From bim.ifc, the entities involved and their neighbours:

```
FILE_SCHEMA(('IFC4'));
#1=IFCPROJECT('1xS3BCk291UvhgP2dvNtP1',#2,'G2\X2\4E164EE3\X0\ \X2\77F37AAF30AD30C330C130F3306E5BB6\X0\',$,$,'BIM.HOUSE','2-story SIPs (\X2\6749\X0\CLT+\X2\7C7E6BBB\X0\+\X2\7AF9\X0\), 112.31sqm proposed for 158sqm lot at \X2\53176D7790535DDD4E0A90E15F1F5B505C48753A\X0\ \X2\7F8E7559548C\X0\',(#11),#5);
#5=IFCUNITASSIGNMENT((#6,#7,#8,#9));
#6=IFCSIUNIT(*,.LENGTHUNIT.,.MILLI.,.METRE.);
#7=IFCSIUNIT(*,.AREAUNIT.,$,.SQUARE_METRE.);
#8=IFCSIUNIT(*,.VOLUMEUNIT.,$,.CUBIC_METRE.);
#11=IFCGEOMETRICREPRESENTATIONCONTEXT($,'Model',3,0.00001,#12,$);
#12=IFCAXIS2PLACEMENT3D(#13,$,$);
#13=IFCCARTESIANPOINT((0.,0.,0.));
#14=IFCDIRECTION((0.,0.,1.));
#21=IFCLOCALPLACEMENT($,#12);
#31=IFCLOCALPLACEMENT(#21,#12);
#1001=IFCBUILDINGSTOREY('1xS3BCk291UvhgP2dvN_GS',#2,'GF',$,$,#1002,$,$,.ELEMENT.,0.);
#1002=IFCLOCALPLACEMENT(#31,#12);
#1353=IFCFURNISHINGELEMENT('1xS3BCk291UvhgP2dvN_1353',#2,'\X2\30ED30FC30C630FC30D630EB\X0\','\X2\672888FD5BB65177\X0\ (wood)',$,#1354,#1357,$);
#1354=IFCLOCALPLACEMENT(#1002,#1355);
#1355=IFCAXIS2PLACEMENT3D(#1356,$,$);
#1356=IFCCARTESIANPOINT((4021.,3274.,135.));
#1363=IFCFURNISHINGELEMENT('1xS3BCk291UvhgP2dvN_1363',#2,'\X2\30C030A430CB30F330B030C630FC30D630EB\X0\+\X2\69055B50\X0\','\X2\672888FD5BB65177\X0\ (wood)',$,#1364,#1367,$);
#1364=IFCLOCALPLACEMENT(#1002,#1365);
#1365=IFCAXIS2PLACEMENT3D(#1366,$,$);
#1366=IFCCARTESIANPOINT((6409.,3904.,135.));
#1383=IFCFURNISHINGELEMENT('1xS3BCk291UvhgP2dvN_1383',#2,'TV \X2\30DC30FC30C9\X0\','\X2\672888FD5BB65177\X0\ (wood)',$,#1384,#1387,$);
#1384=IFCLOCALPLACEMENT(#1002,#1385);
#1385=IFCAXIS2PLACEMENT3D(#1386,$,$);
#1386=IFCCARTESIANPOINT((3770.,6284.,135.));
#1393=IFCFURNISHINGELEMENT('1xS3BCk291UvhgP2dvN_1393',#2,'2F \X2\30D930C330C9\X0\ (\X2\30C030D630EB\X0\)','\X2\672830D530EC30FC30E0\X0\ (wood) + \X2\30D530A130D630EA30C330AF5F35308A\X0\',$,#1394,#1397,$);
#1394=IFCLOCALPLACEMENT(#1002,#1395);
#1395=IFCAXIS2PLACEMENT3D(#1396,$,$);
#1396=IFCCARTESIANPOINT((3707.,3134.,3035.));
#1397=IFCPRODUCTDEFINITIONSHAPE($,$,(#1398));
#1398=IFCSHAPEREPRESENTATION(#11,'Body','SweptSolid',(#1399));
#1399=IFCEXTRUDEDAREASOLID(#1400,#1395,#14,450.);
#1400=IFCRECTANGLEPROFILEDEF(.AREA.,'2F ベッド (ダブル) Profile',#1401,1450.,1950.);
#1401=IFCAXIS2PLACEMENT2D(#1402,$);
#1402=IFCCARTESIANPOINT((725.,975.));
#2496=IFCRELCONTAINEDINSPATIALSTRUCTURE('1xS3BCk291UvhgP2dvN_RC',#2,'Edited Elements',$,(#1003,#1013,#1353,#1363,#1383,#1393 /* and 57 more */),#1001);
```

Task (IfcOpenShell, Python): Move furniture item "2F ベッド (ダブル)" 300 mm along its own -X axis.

```python
import ifcopenshell
import ifcopenshell.api.geometry
import ifcopenshell.util.placement

model = ifcopenshell.open("bim.ifc")

item = model.by_guid("1xS3BCk291UvhgP2dvN_1393")
matrix = ifcopenshell.util.placement.get_local_placement(item.ObjectPlacement)
matrix[:3, 3] -= matrix[:3, 0] * 300.0
ifcopenshell.api.geometry.edit_object_placement(model, product=item, matrix=matrix, is_si=False)

print(ifcopenshell.util.placement.get_local_placement(item.ObjectPlacement).round(3) + 0.0)

model.write("bim-out.ifc")
```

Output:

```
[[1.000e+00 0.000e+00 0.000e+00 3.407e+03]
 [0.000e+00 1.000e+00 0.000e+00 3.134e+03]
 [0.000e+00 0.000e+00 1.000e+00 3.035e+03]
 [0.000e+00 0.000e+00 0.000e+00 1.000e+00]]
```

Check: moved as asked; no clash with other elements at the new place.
